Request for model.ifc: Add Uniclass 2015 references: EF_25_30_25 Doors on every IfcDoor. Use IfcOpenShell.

First a look at what the model holds.

```python
import ifcopenshell

model = ifcopenshell.open("model.ifc")
print(model.schema)
print("classifications:", [c.Name for c in model.by_type("IfcClassification")])
for ifc_class in ("IfcDoor", "IfcRoof", "IfcStair", "IfcWall", "IfcWindow"):
    print(ifc_class, len(model.by_type(ifc_class)))
```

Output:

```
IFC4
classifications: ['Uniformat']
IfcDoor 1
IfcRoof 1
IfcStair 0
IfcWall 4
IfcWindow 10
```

```python
import ifcopenshell
import ifcopenshell.api.classification

model = ifcopenshell.open("model.ifc")

system = ifcopenshell.api.classification.add_classification(model, classification="Uniclass 2015")

codes = {
    "IfcDoor": ("EF_25_30_25", "Doors"),
}
for ifc_class, (code, name) in codes.items():
    products = model.by_type(ifc_class)
    ifcopenshell.api.classification.add_reference(
        model, products=products, classification=system, identification=code, name=name
    )
    print(code, len(products))

model.write("model_rev.ifc")
```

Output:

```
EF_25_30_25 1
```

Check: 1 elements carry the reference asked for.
